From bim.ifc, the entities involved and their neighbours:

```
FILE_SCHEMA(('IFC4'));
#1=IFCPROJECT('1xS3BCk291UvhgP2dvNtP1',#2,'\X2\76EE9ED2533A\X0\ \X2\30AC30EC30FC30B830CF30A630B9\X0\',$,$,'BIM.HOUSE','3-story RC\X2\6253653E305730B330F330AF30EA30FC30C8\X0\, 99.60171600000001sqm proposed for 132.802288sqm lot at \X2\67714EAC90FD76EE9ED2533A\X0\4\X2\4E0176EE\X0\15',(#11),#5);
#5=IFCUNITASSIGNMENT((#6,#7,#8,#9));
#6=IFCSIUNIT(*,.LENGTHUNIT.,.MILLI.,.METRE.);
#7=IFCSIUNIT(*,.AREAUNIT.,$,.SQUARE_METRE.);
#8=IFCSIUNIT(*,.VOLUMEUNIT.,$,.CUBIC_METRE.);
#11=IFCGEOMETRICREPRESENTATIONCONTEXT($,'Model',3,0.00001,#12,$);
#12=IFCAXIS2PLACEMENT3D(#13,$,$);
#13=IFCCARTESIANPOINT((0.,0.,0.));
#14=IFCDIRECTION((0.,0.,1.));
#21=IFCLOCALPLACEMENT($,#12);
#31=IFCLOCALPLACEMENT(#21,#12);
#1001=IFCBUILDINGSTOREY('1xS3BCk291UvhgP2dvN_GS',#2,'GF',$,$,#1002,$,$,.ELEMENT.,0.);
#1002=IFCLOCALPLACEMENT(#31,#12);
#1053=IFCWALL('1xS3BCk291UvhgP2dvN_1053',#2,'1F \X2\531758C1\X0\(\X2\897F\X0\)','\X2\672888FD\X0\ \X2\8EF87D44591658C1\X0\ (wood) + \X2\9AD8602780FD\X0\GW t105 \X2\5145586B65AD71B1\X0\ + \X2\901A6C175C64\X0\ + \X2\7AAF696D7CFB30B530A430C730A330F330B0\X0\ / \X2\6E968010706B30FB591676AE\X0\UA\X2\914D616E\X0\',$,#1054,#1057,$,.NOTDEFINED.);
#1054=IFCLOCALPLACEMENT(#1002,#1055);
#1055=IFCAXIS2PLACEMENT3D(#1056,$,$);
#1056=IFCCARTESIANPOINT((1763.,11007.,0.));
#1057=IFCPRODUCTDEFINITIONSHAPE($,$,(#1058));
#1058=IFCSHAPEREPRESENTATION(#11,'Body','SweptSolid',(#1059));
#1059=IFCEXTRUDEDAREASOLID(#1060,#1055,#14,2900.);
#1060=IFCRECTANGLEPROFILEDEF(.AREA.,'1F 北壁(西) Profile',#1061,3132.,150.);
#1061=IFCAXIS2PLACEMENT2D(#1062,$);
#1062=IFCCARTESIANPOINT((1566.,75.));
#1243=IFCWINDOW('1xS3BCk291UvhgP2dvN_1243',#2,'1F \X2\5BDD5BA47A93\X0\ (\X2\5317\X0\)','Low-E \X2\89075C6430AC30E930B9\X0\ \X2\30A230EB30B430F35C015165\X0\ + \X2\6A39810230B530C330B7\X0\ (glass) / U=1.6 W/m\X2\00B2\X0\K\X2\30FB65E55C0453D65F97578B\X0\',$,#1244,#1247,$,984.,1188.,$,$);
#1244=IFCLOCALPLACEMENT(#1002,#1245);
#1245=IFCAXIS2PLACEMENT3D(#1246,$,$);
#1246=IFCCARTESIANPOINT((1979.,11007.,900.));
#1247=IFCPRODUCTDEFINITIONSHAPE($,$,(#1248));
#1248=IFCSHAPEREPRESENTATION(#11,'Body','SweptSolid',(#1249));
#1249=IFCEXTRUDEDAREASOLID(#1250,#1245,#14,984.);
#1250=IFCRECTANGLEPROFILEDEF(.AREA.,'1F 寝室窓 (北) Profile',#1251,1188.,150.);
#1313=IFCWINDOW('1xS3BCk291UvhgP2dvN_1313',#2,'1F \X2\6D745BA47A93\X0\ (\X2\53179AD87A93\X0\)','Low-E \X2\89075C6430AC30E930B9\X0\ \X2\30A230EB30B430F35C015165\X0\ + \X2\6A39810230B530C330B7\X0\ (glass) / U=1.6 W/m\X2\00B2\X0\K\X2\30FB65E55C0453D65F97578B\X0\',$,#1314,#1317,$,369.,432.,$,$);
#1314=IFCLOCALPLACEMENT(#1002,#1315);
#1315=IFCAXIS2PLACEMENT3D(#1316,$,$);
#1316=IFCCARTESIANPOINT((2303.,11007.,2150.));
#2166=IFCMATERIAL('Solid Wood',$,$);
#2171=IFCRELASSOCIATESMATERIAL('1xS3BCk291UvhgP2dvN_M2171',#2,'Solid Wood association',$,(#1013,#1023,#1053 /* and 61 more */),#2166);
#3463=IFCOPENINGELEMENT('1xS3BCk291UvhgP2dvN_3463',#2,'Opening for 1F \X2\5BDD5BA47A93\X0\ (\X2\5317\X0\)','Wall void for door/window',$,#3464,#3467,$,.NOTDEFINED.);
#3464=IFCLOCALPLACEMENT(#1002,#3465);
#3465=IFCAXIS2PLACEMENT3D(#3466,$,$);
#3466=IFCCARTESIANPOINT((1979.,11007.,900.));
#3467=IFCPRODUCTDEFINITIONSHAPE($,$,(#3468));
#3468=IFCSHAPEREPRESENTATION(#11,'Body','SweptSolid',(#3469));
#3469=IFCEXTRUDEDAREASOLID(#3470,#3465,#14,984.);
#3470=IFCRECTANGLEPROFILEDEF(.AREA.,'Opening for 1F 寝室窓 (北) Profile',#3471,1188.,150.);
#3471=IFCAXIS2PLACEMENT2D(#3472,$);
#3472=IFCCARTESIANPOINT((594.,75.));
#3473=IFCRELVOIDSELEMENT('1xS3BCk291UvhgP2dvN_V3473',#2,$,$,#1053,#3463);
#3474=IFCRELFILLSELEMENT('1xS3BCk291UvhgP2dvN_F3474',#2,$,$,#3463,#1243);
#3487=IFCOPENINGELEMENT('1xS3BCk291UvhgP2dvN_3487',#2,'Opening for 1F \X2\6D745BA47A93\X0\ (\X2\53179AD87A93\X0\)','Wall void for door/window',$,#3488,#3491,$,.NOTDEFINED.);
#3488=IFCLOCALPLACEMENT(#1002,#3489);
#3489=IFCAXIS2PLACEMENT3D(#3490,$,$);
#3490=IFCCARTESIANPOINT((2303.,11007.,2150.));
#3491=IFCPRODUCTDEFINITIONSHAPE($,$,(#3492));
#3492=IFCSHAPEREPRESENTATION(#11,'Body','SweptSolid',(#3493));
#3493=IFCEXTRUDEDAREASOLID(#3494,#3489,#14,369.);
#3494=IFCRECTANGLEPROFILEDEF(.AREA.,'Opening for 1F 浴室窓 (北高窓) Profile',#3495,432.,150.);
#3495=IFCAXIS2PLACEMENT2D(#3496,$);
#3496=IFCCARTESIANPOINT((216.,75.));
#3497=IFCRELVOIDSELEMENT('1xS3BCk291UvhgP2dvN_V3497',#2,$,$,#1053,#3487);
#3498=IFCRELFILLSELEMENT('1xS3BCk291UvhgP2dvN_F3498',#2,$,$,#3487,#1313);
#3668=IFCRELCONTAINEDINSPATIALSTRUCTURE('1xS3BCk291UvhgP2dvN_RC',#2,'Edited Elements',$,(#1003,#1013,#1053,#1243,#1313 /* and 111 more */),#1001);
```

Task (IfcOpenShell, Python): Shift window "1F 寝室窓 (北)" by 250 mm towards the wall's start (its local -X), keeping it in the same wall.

```python
import ifcopenshell
import ifcopenshell.api.geometry
import ifcopenshell.util.placement

model = ifcopenshell.open("bim.ifc")

window = model.by_guid("1xS3BCk291UvhgP2dvN_1243")
opening = window.FillsVoids[0].RelatingOpeningElement
wall = opening.VoidsElements[0].RelatingBuildingElement

wall_matrix = ifcopenshell.util.placement.get_local_placement(wall.ObjectPlacement)
shift = wall_matrix[:3, 0] * -250.0
before = ifcopenshell.util.placement.get_local_placement(window.ObjectPlacement)[:3, 3].copy()

# The window is not placed relative to its opening, so move both.
for product in (opening, window):
    matrix = ifcopenshell.util.placement.get_local_placement(product.ObjectPlacement)
    matrix[:3, 3] += shift
    ifcopenshell.api.geometry.edit_object_placement(model, product=product, matrix=matrix, is_si=False)

after = ifcopenshell.util.placement.get_local_placement(window.ObjectPlacement)[:3, 3]
print("window moved by", (after - before).round(3) + 0.0)

model.write("bim_v2.ifc")
```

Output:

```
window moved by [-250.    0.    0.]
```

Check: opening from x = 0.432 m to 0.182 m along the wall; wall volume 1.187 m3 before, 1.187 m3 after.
